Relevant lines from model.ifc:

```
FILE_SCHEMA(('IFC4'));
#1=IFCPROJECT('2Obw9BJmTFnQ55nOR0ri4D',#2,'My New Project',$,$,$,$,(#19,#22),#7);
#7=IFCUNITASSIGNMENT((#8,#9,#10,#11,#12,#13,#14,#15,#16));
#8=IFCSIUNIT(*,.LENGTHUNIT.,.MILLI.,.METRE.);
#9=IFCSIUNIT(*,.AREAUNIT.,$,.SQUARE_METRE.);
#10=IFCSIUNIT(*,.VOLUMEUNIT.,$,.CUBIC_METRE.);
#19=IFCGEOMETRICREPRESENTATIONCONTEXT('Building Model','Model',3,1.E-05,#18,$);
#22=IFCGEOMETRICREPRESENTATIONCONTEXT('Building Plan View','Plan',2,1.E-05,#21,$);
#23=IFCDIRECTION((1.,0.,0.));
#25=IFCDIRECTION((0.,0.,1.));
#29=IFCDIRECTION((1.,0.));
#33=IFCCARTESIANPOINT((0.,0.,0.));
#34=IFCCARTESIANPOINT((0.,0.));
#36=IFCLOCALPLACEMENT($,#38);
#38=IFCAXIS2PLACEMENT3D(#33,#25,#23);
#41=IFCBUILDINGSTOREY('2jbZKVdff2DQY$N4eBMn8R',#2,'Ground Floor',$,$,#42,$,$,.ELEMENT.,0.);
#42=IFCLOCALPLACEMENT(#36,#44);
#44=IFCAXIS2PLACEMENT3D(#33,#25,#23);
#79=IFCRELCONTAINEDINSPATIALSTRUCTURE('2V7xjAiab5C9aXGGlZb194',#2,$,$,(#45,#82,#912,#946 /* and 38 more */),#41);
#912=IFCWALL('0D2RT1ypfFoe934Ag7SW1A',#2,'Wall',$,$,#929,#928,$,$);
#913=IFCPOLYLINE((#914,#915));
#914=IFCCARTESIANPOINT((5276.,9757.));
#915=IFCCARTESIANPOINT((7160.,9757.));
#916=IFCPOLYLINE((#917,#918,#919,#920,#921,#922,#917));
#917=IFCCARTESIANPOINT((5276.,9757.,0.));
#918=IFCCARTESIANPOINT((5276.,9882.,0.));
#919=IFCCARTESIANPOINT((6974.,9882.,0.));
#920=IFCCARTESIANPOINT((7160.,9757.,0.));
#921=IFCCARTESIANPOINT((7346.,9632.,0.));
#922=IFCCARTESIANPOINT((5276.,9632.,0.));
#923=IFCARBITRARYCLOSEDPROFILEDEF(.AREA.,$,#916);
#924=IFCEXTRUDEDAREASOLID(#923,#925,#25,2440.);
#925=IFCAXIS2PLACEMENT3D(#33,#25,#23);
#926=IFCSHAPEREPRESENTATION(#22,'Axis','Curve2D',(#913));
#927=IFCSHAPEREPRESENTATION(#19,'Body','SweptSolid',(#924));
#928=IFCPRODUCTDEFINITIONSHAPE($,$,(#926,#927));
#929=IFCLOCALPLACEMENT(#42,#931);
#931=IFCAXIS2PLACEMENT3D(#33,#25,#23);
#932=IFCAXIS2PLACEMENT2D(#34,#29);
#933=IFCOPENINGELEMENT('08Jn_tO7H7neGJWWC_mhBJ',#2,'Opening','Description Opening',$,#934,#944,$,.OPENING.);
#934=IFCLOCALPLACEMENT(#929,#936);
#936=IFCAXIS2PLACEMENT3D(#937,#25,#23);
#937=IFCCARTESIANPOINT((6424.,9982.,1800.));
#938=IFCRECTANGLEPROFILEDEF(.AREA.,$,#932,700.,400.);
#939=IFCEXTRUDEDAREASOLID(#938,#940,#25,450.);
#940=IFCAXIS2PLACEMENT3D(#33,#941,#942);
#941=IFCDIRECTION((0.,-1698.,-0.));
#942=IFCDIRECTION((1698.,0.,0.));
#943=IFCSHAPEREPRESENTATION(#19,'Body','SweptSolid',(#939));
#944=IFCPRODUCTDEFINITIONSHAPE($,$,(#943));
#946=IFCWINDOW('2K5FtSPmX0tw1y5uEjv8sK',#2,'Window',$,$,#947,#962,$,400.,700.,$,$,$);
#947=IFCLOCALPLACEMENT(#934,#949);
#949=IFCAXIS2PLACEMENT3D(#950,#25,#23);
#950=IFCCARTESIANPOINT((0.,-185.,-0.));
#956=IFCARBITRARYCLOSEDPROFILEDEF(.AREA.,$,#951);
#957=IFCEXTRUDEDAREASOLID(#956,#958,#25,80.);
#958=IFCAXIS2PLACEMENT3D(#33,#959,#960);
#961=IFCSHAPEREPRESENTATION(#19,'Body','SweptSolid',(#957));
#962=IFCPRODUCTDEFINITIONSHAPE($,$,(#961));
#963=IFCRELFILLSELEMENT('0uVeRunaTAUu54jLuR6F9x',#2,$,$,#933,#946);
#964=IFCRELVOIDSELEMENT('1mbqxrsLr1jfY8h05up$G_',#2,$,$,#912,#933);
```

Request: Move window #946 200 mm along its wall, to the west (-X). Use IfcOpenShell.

```python
import ifcopenshell
import ifcopenshell.api.geometry
import ifcopenshell.util.placement
import ifcopenshell.util.unit

model = ifcopenshell.open("model.ifc")
unit_scale = ifcopenshell.util.unit.calculate_unit_scale(model)

window = model.by_guid("2K5FtSPmX0tw1y5uEjv8sK")
opening = window.FillsVoids[0].RelatingOpeningElement
wall = opening.VoidsElements[0].RelatingBuildingElement

wall_matrix = ifcopenshell.util.placement.get_local_placement(wall.ObjectPlacement)
shift = wall_matrix[:3, 0] * -0.2 / unit_scale
before = ifcopenshell.util.placement.get_local_placement(window.ObjectPlacement)[:3, 3].copy()

# The window is placed relative to its opening, so it follows when the opening moves.
matrix = ifcopenshell.util.placement.get_local_placement(opening.ObjectPlacement)
matrix[:3, 3] += shift
ifcopenshell.api.geometry.edit_object_placement(
    model, product=opening, matrix=matrix, is_si=False, should_transform_children=True
)

after = ifcopenshell.util.placement.get_local_placement(window.ObjectPlacement)[:3, 3]
print("window moved by", (after - before).round(3) + 0.0)

model.write("model_rev.ifc")
```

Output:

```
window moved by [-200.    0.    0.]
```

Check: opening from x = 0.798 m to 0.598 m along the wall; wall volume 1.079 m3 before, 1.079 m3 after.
